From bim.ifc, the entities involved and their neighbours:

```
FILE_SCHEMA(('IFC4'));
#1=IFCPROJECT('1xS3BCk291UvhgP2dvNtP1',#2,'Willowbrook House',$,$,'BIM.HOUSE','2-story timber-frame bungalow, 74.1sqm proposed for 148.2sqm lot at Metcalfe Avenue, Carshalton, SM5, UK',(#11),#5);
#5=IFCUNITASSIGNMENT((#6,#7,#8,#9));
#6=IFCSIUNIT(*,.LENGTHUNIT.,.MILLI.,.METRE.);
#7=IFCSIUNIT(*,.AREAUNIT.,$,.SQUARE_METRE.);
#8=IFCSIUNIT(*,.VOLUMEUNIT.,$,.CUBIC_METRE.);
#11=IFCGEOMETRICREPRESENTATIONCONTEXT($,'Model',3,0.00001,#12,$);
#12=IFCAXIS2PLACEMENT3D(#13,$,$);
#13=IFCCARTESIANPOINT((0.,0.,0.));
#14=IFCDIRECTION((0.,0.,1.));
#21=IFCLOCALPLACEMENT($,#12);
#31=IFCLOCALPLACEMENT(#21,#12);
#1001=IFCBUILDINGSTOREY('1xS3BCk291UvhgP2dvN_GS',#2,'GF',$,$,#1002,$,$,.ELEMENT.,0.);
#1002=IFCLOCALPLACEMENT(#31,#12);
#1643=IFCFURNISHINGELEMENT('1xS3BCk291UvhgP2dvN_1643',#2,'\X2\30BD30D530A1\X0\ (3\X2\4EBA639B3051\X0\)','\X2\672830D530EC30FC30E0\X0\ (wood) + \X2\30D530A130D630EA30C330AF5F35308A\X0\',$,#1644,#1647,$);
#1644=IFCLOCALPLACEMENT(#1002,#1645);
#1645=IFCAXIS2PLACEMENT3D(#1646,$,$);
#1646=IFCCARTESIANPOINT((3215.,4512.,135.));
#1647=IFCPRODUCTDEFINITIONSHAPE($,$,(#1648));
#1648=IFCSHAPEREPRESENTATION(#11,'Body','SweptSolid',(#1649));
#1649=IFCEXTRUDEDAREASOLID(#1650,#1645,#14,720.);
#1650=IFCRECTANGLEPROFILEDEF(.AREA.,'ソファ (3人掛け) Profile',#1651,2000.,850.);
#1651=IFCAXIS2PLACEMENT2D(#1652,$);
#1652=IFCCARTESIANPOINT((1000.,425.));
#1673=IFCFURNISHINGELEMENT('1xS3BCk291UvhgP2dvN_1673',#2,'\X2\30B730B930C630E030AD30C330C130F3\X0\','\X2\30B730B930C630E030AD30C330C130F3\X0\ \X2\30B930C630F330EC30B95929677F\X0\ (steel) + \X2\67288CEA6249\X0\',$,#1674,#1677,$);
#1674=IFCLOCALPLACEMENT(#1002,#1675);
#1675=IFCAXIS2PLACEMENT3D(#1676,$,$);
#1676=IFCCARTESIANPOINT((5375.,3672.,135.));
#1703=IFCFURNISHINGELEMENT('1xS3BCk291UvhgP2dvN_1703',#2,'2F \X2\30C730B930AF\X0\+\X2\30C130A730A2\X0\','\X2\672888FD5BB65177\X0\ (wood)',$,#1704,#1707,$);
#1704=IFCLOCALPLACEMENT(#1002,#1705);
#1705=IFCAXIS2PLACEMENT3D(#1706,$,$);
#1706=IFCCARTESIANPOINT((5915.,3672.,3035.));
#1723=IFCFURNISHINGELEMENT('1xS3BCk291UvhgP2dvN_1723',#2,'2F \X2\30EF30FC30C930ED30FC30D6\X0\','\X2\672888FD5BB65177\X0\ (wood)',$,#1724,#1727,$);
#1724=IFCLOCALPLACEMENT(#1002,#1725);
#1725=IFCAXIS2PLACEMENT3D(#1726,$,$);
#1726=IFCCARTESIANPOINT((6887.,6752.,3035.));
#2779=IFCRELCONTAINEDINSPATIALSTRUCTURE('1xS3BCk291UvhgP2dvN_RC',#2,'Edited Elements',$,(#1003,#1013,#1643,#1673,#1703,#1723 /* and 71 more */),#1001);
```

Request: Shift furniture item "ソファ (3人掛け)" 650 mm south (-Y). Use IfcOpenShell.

```python
import ifcopenshell
import ifcopenshell.api.geometry
import ifcopenshell.util.placement
import ifcopenshell.util.unit

model = ifcopenshell.open("bim.ifc")
unit_scale = ifcopenshell.util.unit.calculate_unit_scale(model)

item = model.by_guid("1xS3BCk291UvhgP2dvN_1643")
matrix = ifcopenshell.util.placement.get_local_placement(item.ObjectPlacement)
matrix[1, 3] -= 0.65 / unit_scale
ifcopenshell.api.geometry.edit_object_placement(model, product=item, matrix=matrix, is_si=False)

print(ifcopenshell.util.placement.get_local_placement(item.ObjectPlacement).round(3) + 0.0)

model.write("bim_v2.ifc")
```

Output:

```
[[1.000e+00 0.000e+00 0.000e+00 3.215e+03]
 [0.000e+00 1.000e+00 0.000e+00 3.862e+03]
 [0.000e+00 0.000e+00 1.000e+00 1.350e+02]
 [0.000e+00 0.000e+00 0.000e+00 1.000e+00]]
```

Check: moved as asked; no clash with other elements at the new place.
